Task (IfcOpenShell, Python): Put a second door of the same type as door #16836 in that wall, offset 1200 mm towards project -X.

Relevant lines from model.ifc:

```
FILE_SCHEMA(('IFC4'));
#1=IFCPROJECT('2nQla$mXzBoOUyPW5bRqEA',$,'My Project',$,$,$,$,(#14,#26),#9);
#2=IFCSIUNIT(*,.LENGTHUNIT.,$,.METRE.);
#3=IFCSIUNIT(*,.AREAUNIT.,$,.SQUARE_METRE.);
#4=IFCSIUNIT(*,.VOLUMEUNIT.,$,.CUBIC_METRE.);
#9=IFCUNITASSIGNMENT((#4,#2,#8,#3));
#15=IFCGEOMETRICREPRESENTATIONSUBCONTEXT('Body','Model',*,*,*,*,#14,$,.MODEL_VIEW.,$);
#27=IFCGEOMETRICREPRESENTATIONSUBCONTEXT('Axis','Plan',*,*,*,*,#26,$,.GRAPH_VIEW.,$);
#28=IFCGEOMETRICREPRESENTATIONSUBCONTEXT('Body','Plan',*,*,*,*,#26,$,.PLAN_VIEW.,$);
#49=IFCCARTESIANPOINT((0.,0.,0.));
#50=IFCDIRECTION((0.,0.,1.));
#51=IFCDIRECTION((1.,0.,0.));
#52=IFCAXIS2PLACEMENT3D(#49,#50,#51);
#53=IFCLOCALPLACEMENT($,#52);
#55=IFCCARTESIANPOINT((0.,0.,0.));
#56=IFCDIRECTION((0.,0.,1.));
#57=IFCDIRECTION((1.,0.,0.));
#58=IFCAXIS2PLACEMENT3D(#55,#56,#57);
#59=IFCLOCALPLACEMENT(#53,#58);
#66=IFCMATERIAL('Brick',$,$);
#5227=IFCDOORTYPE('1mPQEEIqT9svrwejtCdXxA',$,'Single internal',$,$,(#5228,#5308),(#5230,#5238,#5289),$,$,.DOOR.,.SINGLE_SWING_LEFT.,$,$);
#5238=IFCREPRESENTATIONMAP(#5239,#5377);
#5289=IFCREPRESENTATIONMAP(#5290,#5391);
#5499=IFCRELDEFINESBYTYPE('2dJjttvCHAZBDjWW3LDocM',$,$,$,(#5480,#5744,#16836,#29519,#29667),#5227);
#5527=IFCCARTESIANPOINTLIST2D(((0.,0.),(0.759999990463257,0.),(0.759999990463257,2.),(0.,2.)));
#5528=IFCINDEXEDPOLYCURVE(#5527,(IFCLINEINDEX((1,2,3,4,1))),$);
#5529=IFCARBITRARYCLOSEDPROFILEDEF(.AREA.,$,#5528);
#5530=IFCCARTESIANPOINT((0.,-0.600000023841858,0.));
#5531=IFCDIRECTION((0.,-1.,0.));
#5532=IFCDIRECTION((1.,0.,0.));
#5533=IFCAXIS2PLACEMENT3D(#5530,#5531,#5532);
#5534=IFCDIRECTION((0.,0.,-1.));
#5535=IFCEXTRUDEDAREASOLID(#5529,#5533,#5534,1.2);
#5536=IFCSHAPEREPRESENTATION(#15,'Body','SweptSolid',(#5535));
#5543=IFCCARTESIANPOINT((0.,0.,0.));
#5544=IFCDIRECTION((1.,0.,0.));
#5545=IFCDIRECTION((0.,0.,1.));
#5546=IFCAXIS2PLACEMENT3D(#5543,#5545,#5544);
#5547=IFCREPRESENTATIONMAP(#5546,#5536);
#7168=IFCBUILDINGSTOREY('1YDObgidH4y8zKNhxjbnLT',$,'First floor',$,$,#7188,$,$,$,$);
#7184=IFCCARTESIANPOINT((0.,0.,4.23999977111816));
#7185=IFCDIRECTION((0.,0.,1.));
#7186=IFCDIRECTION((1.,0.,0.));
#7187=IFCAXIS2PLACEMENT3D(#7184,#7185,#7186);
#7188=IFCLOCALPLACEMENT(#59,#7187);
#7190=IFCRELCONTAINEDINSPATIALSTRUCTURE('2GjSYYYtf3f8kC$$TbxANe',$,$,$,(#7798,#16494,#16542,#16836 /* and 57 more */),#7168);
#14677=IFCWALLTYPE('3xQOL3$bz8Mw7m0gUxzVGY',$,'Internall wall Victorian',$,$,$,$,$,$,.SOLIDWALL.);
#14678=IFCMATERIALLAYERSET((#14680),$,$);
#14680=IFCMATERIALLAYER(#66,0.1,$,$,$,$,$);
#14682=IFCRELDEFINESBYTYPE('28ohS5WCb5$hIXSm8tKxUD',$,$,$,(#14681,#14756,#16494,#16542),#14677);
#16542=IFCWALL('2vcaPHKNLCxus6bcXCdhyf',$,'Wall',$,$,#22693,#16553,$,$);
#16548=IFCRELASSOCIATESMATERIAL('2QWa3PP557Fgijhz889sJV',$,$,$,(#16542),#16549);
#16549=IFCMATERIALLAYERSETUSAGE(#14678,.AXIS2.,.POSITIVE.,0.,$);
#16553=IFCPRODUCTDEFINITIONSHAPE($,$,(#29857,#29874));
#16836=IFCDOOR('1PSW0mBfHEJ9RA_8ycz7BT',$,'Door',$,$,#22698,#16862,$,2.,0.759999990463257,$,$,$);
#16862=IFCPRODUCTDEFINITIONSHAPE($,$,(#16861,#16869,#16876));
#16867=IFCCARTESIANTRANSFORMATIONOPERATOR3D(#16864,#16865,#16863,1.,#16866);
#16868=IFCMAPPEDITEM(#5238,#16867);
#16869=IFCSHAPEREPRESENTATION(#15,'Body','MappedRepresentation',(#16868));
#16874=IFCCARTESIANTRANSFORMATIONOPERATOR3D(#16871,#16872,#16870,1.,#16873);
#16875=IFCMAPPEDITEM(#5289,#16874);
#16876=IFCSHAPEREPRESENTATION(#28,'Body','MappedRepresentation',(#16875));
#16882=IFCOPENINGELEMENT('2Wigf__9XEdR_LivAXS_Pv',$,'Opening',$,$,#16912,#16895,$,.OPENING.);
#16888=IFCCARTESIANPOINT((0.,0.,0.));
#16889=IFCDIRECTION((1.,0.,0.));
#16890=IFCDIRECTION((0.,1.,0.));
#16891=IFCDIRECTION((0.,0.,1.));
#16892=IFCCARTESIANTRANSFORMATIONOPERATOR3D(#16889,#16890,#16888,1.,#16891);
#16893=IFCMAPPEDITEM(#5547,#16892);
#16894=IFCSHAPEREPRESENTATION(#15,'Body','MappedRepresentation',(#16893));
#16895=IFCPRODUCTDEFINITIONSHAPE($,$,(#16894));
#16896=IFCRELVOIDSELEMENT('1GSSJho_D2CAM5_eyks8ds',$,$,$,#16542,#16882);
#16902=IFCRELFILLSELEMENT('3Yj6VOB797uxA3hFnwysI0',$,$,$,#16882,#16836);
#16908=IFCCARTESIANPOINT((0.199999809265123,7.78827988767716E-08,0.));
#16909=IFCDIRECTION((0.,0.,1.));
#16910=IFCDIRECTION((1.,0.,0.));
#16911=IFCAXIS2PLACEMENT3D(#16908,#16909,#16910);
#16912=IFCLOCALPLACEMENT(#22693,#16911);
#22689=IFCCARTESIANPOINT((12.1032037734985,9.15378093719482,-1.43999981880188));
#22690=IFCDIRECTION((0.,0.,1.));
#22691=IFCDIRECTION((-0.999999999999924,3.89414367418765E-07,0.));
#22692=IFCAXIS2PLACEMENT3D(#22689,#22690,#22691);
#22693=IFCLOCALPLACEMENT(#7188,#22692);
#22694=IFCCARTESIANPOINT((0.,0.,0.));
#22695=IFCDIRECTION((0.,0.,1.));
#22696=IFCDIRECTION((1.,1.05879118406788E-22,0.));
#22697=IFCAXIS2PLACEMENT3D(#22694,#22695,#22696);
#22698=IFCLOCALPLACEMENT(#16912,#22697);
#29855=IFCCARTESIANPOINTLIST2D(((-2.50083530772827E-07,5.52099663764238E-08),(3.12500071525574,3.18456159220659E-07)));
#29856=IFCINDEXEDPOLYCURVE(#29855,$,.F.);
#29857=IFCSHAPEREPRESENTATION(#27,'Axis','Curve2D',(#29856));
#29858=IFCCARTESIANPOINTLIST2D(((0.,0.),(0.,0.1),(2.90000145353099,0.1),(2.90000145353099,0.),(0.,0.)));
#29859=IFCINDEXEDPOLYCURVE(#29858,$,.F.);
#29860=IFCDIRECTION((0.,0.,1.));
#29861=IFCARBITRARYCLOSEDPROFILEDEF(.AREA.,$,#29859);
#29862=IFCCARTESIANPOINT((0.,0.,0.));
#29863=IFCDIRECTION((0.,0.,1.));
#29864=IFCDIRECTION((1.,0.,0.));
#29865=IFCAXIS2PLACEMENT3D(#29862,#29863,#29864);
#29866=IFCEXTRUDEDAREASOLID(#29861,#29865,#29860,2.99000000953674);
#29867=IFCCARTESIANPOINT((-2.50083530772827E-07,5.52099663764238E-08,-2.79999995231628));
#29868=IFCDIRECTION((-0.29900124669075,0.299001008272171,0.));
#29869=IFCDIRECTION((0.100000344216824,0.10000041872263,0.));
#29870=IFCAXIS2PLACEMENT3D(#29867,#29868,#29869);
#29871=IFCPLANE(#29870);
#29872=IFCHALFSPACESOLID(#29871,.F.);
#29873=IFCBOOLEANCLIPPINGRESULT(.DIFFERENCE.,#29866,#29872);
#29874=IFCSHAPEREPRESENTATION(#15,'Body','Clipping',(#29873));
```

```python
import ifcopenshell
import ifcopenshell.api.feature
import ifcopenshell.api.geometry
import ifcopenshell.api.root
import ifcopenshell.geom
import ifcopenshell.util.element
import ifcopenshell.util.placement
import ifcopenshell.util.shape
import ifcopenshell.util.unit

model = ifcopenshell.open("model.ifc")
unit_scale = ifcopenshell.util.unit.calculate_unit_scale(model)
settings = ifcopenshell.geom.settings()


def volume(element):
    """Net volume in cubic metres, openings subtracted."""
    shape = ifcopenshell.geom.create_shape(settings, element)
    return ifcopenshell.util.shape.get_volume(shape.geometry)


door = model.by_guid("1PSW0mBfHEJ9RA_8ycz7BT")
opening = door.FillsVoids[0].RelatingOpeningElement
wall = opening.VoidsElements[0].RelatingBuildingElement
before = volume(wall)
shift = ifcopenshell.util.placement.get_local_placement(wall.ObjectPlacement)[:3, 0] * 1.2 / unit_scale

# copy_class copies the void relationship, type, container and properties, but no geometry.
new_opening = ifcopenshell.api.root.copy_class(model, product=opening)
new_opening.Representation = ifcopenshell.util.element.copy_deep(
    model, opening.Representation, exclude=["IfcGeometricRepresentationContext", "IfcRepresentationMap"]
)
new_door = ifcopenshell.api.root.copy_class(model, product=door)
new_door.Representation = ifcopenshell.util.element.copy_deep(
    model, door.Representation, exclude=["IfcGeometricRepresentationContext", "IfcRepresentationMap"]
)
ifcopenshell.api.feature.add_filling(model, opening=new_opening, element=new_door)

for old, new in ((opening, new_opening), (door, new_door)):
    matrix = ifcopenshell.util.placement.get_local_placement(old.ObjectPlacement)
    matrix[:3, 3] += shift
    ifcopenshell.api.geometry.edit_object_placement(model, product=new, matrix=matrix, is_si=False)

after = volume(wall)

print(f"wall volume {before:.3f} -> {after:.3f} m3")

model.write("model_updated.ifc")
```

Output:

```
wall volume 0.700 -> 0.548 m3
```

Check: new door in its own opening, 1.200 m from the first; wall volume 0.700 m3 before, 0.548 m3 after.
